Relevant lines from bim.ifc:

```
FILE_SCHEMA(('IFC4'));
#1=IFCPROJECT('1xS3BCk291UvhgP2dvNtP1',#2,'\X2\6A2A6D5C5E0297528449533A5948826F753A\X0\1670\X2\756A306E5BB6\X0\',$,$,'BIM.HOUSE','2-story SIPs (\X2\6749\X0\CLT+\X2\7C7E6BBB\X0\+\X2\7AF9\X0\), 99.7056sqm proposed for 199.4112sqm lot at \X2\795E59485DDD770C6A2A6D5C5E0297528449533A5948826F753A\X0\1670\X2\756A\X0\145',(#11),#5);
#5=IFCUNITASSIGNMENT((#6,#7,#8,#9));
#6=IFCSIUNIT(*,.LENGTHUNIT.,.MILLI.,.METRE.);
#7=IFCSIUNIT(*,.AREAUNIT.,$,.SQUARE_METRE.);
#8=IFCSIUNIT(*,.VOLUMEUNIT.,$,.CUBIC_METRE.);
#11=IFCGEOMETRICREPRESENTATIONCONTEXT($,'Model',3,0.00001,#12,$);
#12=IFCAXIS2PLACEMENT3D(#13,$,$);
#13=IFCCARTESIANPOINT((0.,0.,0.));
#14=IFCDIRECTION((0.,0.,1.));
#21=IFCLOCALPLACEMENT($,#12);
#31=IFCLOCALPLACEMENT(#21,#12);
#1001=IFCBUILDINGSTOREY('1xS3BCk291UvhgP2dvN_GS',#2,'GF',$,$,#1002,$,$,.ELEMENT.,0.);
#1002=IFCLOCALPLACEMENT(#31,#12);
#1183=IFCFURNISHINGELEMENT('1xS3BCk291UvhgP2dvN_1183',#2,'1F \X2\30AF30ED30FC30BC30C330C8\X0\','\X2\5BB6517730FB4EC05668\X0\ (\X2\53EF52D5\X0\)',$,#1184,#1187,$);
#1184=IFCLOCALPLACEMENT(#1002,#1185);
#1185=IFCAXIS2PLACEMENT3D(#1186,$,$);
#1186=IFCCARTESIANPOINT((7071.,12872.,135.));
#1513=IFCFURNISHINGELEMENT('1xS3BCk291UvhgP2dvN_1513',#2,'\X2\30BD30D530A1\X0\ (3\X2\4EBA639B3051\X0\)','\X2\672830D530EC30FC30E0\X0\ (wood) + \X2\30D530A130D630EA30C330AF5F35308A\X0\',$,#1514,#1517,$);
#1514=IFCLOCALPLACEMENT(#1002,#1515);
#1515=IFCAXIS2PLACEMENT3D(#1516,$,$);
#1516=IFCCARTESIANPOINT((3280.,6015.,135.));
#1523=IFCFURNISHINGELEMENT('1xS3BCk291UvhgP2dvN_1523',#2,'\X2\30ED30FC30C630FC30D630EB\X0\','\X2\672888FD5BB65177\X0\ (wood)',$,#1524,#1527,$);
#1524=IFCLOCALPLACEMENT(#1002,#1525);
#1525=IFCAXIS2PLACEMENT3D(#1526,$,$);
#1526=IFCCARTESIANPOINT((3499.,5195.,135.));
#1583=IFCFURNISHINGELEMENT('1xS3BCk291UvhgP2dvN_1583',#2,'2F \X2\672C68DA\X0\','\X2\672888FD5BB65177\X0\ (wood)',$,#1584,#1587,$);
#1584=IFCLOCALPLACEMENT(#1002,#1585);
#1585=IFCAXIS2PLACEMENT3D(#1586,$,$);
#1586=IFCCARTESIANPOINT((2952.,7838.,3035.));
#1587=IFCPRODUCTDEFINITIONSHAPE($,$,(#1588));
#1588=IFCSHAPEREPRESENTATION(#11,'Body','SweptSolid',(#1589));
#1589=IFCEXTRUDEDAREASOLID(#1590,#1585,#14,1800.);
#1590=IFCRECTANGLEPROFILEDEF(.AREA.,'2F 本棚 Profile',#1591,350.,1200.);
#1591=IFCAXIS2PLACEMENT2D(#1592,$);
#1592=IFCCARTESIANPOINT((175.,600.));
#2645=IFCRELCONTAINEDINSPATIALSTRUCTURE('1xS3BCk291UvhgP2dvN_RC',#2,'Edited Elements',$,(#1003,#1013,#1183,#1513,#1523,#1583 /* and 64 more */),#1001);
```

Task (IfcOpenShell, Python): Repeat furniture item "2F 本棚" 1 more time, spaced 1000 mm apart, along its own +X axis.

```python
import ifcopenshell
import ifcopenshell.api.geometry
import ifcopenshell.api.root
import ifcopenshell.util.element
import ifcopenshell.util.placement

model = ifcopenshell.open("bim.ifc")


def reuse_history(source, copy):
    """copy_class also copies each property set's owner history, people and application; keep the originals."""
    for rel in copy.IsDefinedBy:
        if rel.is_a("IfcRelDefinesByProperties") and (history := rel.RelatingPropertyDefinition.OwnerHistory):
            rel.RelatingPropertyDefinition.OwnerHistory = source.OwnerHistory
            ifcopenshell.util.element.remove_deep2(model, history)


source = model.by_id(1583)
base = ifcopenshell.util.placement.get_local_placement(source.ObjectPlacement)
step = base[:3, 0] * 1000.0

for i in range(1, 2):
    copy = ifcopenshell.api.root.copy_class(model, product=source)
    copy.Representation = ifcopenshell.util.element.copy_deep(
        model, source.Representation, exclude=["IfcGeometricRepresentationContext", "IfcRepresentationMap"]
    )
    reuse_history(source, copy)
    matrix = base.copy()
    matrix[:3, 3] += i * step
    print("added at", matrix[:3, 3].round(3) + 0.0)
    ifcopenshell.api.geometry.edit_object_placement(model, product=copy, matrix=matrix, is_si=False)

model.write("bim_rev.ifc")
```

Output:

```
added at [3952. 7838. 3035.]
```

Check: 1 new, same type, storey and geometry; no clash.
